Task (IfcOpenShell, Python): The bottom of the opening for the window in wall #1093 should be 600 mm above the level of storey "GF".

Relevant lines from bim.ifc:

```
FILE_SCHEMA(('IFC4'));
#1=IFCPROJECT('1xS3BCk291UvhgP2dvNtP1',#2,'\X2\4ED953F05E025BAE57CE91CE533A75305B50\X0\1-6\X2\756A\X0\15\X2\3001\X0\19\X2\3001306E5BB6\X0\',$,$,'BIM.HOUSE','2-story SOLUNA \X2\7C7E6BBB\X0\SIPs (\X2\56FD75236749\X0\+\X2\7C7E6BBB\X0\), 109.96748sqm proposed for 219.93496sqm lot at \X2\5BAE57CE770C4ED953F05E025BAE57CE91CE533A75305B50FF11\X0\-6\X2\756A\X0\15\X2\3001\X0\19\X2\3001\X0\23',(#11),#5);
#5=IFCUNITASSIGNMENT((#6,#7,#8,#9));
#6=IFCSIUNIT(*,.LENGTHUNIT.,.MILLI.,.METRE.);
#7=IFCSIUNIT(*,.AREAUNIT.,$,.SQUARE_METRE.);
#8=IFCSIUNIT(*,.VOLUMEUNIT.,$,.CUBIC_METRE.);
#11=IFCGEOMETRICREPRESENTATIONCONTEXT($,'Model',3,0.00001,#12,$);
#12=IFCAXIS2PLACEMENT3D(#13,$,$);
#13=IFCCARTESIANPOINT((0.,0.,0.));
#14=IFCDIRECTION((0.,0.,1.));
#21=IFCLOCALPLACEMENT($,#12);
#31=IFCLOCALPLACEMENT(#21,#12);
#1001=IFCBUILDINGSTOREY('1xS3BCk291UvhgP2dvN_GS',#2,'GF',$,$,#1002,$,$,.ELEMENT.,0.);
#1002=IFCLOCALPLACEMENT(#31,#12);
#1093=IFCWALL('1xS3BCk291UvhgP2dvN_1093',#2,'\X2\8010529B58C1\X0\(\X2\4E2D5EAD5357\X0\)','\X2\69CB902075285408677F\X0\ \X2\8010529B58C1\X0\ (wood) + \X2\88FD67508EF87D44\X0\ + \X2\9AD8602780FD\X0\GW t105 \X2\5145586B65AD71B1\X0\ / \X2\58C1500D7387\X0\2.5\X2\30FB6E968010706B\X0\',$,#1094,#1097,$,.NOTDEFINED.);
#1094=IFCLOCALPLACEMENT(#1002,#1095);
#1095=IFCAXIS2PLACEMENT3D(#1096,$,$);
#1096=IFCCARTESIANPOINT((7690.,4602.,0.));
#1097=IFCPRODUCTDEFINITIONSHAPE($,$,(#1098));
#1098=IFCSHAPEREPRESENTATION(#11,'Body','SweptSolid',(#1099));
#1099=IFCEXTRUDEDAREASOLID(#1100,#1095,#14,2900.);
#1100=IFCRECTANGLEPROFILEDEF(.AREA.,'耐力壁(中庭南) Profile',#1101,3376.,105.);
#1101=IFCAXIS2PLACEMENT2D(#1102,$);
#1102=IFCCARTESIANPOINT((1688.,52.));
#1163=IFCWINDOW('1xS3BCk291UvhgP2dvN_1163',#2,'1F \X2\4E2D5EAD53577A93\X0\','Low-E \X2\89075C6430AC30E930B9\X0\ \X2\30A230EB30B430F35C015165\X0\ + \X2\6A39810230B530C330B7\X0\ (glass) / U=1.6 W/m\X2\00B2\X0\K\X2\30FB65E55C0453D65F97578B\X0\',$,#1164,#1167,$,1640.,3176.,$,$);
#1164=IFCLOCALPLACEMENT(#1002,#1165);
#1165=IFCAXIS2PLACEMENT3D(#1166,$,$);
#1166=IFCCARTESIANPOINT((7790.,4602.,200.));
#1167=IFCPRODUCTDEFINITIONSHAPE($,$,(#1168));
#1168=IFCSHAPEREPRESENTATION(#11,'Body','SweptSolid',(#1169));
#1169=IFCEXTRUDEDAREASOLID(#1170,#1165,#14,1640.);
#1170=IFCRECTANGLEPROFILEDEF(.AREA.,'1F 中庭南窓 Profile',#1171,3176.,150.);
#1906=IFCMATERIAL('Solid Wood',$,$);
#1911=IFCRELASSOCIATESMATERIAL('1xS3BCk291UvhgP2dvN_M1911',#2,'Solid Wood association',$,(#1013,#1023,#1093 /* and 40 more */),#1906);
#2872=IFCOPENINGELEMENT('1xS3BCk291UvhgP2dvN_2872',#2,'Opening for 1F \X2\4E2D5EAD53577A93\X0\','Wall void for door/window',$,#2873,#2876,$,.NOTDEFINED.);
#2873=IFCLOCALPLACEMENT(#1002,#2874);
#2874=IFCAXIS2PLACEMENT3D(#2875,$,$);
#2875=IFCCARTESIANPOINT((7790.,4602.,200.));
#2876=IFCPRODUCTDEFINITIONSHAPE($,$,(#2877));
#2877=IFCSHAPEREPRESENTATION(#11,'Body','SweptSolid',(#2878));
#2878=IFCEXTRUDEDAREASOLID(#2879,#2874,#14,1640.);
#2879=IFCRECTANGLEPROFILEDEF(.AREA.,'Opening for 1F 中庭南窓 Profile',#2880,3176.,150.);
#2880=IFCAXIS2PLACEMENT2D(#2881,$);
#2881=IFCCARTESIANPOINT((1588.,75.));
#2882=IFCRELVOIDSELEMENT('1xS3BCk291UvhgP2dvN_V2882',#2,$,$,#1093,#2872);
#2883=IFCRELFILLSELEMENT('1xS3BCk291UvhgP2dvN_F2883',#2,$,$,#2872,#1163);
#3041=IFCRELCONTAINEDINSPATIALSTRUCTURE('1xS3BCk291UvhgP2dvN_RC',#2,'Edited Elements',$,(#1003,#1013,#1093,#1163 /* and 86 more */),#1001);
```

```python
import numpy as np
import ifcopenshell
import ifcopenshell.api.geometry
import ifcopenshell.geom
import ifcopenshell.util.element
import ifcopenshell.util.placement
import ifcopenshell.util.shape
import ifcopenshell.util.unit

model = ifcopenshell.open("bim.ifc")
unit_scale = ifcopenshell.util.unit.calculate_unit_scale(model)

window = model.by_guid("1xS3BCk291UvhgP2dvN_1163")
opening = window.FillsVoids[0].RelatingOpeningElement
storey = ifcopenshell.util.element.get_container(window, ifc_class="IfcBuildingStorey")
level = ifcopenshell.util.placement.get_local_placement(storey.ObjectPlacement)[2, 3]

# The opening's origin need not be at the sill, so measure its lowest point.
shape = ifcopenshell.geom.create_shape(ifcopenshell.geom.settings(), opening)
bottom = ifcopenshell.util.shape.get_shape_bottom_elevation(shape, shape.geometry) / unit_scale
dz = level + 0.6 / unit_scale - bottom

shift = np.array([0.0, 0.0, dz])
# The window is not placed relative to its opening, so move both.
for product in (opening, window):
    matrix = ifcopenshell.util.placement.get_local_placement(product.ObjectPlacement)
    matrix[:3, 3] += shift
    ifcopenshell.api.geometry.edit_object_placement(model, product=product, matrix=matrix, is_si=False)

print(f"moved by {dz * unit_scale:+.3f} m")

model.write("bim-out.ifc")
```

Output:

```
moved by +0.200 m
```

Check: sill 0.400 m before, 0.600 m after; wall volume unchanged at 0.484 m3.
